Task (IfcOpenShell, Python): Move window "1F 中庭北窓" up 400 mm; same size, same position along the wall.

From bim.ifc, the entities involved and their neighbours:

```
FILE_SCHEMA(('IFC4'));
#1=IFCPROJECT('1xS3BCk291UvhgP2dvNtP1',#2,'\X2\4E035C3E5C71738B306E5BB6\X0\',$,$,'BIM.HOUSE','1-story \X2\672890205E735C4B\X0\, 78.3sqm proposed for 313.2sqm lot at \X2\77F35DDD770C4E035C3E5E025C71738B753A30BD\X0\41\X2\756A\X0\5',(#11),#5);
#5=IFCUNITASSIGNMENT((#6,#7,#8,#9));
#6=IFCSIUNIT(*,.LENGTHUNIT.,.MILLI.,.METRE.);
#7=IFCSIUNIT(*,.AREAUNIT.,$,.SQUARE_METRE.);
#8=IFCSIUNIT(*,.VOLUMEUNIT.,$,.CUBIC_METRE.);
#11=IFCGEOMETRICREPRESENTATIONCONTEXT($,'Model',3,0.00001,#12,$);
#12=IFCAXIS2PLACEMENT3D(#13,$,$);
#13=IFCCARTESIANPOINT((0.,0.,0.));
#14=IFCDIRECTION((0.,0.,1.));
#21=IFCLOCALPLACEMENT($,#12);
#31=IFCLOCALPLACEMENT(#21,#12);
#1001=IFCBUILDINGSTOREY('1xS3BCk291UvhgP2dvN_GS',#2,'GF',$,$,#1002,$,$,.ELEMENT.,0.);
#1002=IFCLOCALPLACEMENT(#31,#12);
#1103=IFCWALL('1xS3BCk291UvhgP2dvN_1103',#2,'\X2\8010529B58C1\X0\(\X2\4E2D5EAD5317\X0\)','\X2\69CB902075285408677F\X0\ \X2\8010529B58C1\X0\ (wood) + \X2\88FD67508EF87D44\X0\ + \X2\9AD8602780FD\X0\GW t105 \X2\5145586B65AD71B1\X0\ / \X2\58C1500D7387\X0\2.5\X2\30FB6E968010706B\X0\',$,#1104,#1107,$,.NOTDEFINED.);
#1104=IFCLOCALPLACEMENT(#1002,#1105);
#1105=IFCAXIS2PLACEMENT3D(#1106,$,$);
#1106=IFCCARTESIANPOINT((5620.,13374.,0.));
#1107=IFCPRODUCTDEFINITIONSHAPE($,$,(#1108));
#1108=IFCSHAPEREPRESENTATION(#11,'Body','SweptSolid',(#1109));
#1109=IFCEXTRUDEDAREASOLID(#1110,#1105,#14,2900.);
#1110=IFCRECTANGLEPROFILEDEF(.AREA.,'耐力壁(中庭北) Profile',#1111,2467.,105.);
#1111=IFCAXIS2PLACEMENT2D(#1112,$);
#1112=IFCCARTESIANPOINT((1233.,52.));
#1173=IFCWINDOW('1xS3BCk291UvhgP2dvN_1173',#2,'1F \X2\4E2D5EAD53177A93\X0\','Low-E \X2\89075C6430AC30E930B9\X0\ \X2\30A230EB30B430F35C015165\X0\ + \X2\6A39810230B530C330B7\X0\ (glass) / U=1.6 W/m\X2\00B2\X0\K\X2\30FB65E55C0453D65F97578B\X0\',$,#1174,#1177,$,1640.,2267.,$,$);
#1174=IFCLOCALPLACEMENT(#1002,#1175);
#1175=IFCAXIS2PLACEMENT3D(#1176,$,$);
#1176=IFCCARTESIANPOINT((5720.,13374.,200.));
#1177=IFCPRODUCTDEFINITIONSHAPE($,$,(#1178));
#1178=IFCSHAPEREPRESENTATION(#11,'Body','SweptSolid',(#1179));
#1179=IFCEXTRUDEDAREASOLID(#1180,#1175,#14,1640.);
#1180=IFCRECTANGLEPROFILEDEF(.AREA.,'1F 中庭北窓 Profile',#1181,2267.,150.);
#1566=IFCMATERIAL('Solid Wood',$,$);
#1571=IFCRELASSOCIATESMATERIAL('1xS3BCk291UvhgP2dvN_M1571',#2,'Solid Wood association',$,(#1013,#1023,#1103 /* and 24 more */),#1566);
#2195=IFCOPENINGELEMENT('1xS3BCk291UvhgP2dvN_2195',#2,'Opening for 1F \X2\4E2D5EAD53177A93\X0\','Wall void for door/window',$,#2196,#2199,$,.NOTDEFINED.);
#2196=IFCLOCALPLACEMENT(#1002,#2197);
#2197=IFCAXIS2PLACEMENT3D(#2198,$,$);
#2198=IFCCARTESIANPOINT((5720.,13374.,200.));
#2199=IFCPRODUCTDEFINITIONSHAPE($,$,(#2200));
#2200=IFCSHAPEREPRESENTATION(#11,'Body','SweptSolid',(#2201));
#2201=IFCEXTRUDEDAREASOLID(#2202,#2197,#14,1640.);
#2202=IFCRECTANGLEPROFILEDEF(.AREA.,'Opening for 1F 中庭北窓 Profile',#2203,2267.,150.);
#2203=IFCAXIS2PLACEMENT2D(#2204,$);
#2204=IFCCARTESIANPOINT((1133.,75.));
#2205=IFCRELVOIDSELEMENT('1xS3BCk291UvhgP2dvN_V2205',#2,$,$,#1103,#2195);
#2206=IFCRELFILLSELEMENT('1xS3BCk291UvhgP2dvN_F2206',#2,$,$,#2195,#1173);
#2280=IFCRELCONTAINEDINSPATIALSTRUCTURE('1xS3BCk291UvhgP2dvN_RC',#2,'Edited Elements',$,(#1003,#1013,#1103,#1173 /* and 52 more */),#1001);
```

```python
import numpy as np
import ifcopenshell
import ifcopenshell.api.geometry
import ifcopenshell.util.placement
import ifcopenshell.util.unit

model = ifcopenshell.open("bim.ifc")
unit_scale = ifcopenshell.util.unit.calculate_unit_scale(model)

window = model.by_id(1173)
opening = window.FillsVoids[0].RelatingOpeningElement
dz = 0.4 / unit_scale

shift = np.array([0.0, 0.0, dz])
# The window is not placed relative to its opening, so move both.
for product in (opening, window):
    matrix = ifcopenshell.util.placement.get_local_placement(product.ObjectPlacement)
    matrix[:3, 3] += shift
    ifcopenshell.api.geometry.edit_object_placement(model, product=product, matrix=matrix, is_si=False)

print(f"moved by {dz * unit_scale:+.3f} m")

model.write("bim_updated.ifc")
```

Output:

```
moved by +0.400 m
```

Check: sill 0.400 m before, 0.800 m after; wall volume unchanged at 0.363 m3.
